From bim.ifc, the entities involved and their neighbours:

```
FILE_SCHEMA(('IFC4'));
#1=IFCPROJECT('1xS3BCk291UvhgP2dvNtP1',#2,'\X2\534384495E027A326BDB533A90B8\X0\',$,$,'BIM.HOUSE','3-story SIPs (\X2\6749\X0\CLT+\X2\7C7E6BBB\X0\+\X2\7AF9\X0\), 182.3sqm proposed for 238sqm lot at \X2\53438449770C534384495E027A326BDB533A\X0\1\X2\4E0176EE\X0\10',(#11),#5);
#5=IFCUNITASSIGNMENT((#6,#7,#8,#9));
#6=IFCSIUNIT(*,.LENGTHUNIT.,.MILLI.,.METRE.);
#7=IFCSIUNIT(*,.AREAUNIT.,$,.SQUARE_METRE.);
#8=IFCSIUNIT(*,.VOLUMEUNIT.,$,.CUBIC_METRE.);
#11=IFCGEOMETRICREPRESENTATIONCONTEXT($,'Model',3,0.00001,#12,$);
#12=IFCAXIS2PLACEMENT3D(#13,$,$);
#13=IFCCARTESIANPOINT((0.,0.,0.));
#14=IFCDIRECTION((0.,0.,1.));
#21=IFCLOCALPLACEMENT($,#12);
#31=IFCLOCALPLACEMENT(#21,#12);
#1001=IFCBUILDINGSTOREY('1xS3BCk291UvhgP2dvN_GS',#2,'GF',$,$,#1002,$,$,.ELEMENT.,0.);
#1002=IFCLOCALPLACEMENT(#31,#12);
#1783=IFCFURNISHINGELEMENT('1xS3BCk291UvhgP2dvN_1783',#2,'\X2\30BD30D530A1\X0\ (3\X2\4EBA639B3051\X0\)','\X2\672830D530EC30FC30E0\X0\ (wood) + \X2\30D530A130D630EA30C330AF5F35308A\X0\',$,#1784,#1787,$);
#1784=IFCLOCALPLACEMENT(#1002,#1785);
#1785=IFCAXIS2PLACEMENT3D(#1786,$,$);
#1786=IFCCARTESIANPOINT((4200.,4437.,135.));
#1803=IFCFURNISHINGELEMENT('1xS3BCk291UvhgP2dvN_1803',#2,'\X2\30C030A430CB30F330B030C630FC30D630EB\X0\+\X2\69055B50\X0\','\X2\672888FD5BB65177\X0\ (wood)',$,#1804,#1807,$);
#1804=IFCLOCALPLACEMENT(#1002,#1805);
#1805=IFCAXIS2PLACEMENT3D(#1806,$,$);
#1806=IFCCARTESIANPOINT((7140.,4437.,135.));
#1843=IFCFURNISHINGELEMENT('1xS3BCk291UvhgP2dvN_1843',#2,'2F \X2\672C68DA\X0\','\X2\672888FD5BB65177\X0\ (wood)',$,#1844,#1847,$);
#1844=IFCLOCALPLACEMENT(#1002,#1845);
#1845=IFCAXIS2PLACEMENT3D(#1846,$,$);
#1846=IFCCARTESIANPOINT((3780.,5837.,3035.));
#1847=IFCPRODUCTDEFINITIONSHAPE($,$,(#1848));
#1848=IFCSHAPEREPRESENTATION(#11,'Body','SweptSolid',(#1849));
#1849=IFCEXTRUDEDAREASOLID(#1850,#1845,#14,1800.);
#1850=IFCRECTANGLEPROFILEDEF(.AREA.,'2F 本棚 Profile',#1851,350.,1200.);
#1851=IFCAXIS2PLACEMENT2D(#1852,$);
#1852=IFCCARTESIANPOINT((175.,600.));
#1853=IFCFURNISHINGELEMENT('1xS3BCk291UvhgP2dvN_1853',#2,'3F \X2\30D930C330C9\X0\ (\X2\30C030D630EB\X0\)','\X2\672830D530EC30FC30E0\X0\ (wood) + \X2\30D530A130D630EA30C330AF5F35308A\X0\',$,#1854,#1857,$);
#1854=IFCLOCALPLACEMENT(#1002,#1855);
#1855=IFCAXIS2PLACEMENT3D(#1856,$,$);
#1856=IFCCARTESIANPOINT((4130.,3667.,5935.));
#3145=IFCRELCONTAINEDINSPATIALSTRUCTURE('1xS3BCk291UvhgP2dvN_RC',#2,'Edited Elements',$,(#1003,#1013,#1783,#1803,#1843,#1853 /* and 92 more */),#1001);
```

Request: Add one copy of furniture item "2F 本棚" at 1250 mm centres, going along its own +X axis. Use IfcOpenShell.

```python
import ifcopenshell
import ifcopenshell.api.geometry
import ifcopenshell.api.root
import ifcopenshell.util.element
import ifcopenshell.util.placement

model = ifcopenshell.open("bim.ifc")


def reuse_history(source, copy):
    """copy_class also copies each property set's owner history, people and application; keep the originals."""
    for rel in copy.IsDefinedBy:
        if rel.is_a("IfcRelDefinesByProperties") and (history := rel.RelatingPropertyDefinition.OwnerHistory):
            rel.RelatingPropertyDefinition.OwnerHistory = source.OwnerHistory
            ifcopenshell.util.element.remove_deep2(model, history)


source = model.by_guid("1xS3BCk291UvhgP2dvN_1843")
base = ifcopenshell.util.placement.get_local_placement(source.ObjectPlacement)
step = base[:3, 0] * 1250.0

for i in range(1, 2):
    copy = ifcopenshell.api.root.copy_class(model, product=source)
    copy.Representation = ifcopenshell.util.element.copy_deep(
        model, source.Representation, exclude=["IfcGeometricRepresentationContext", "IfcRepresentationMap"]
    )
    reuse_history(source, copy)
    matrix = base.copy()
    matrix[:3, 3] += i * step
    print("added at", matrix[:3, 3].round(3) + 0.0)
    ifcopenshell.api.geometry.edit_object_placement(model, product=copy, matrix=matrix, is_si=False)

model.write("bim_edited.ifc")
```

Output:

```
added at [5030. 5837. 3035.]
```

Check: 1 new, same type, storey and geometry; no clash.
